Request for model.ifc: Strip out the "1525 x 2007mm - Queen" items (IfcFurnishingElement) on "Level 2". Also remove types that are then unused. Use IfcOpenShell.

First a look at what the model holds.

```python
import ifcopenshell
import ifcopenshell.util.element

model = ifcopenshell.open("model.ifc")
print(model.schema)
storey = next(s for s in model.by_type("IfcBuildingStorey") if s.Name == "Level 2")
furniture = [e for e in ifcopenshell.util.element.get_decomposition(storey) if e.is_a("IfcFurnishingElement")]
seen = {}
for e in furniture:
    element_type = ifcopenshell.util.element.get_type(e)
    name = element_type.Name if element_type not in (None, e) else None
    seen[name] = seen.get(name, 0) + 1
for name, count in sorted(seen.items(), key=str):
    print(count, "x", name)
```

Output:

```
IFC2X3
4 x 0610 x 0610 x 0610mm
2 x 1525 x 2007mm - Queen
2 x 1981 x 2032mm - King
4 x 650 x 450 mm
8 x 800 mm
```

```python
import ifcopenshell
import ifcopenshell.api.root
import ifcopenshell.util.element

model = ifcopenshell.open("model.ifc")

storey = next(s for s in model.by_type("IfcBuildingStorey") if s.Name == "Level 2")
furniture = [e for e in ifcopenshell.util.element.get_decomposition(storey) if e.is_a("IfcFurnishingElement")]
targets = [e for e in furniture if (t := ifcopenshell.util.element.get_type(e)) not in (None, e) and t.Name == "1525 x 2007mm - Queen"]
types = {ifcopenshell.util.element.get_type(e) for e in targets} - {None, *targets}

for e in targets:
    ifcopenshell.api.root.remove_product(model, product=e)
print(len(targets), "removed")

unused = [t for t in types if not ifcopenshell.util.element.get_types(t)]
for t in unused:
    ifcopenshell.api.root.remove_product(model, product=t)
print(len(unused), "unused types removed")

model.write("model-out.ifc")
```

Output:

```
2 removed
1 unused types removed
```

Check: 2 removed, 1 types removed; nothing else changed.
